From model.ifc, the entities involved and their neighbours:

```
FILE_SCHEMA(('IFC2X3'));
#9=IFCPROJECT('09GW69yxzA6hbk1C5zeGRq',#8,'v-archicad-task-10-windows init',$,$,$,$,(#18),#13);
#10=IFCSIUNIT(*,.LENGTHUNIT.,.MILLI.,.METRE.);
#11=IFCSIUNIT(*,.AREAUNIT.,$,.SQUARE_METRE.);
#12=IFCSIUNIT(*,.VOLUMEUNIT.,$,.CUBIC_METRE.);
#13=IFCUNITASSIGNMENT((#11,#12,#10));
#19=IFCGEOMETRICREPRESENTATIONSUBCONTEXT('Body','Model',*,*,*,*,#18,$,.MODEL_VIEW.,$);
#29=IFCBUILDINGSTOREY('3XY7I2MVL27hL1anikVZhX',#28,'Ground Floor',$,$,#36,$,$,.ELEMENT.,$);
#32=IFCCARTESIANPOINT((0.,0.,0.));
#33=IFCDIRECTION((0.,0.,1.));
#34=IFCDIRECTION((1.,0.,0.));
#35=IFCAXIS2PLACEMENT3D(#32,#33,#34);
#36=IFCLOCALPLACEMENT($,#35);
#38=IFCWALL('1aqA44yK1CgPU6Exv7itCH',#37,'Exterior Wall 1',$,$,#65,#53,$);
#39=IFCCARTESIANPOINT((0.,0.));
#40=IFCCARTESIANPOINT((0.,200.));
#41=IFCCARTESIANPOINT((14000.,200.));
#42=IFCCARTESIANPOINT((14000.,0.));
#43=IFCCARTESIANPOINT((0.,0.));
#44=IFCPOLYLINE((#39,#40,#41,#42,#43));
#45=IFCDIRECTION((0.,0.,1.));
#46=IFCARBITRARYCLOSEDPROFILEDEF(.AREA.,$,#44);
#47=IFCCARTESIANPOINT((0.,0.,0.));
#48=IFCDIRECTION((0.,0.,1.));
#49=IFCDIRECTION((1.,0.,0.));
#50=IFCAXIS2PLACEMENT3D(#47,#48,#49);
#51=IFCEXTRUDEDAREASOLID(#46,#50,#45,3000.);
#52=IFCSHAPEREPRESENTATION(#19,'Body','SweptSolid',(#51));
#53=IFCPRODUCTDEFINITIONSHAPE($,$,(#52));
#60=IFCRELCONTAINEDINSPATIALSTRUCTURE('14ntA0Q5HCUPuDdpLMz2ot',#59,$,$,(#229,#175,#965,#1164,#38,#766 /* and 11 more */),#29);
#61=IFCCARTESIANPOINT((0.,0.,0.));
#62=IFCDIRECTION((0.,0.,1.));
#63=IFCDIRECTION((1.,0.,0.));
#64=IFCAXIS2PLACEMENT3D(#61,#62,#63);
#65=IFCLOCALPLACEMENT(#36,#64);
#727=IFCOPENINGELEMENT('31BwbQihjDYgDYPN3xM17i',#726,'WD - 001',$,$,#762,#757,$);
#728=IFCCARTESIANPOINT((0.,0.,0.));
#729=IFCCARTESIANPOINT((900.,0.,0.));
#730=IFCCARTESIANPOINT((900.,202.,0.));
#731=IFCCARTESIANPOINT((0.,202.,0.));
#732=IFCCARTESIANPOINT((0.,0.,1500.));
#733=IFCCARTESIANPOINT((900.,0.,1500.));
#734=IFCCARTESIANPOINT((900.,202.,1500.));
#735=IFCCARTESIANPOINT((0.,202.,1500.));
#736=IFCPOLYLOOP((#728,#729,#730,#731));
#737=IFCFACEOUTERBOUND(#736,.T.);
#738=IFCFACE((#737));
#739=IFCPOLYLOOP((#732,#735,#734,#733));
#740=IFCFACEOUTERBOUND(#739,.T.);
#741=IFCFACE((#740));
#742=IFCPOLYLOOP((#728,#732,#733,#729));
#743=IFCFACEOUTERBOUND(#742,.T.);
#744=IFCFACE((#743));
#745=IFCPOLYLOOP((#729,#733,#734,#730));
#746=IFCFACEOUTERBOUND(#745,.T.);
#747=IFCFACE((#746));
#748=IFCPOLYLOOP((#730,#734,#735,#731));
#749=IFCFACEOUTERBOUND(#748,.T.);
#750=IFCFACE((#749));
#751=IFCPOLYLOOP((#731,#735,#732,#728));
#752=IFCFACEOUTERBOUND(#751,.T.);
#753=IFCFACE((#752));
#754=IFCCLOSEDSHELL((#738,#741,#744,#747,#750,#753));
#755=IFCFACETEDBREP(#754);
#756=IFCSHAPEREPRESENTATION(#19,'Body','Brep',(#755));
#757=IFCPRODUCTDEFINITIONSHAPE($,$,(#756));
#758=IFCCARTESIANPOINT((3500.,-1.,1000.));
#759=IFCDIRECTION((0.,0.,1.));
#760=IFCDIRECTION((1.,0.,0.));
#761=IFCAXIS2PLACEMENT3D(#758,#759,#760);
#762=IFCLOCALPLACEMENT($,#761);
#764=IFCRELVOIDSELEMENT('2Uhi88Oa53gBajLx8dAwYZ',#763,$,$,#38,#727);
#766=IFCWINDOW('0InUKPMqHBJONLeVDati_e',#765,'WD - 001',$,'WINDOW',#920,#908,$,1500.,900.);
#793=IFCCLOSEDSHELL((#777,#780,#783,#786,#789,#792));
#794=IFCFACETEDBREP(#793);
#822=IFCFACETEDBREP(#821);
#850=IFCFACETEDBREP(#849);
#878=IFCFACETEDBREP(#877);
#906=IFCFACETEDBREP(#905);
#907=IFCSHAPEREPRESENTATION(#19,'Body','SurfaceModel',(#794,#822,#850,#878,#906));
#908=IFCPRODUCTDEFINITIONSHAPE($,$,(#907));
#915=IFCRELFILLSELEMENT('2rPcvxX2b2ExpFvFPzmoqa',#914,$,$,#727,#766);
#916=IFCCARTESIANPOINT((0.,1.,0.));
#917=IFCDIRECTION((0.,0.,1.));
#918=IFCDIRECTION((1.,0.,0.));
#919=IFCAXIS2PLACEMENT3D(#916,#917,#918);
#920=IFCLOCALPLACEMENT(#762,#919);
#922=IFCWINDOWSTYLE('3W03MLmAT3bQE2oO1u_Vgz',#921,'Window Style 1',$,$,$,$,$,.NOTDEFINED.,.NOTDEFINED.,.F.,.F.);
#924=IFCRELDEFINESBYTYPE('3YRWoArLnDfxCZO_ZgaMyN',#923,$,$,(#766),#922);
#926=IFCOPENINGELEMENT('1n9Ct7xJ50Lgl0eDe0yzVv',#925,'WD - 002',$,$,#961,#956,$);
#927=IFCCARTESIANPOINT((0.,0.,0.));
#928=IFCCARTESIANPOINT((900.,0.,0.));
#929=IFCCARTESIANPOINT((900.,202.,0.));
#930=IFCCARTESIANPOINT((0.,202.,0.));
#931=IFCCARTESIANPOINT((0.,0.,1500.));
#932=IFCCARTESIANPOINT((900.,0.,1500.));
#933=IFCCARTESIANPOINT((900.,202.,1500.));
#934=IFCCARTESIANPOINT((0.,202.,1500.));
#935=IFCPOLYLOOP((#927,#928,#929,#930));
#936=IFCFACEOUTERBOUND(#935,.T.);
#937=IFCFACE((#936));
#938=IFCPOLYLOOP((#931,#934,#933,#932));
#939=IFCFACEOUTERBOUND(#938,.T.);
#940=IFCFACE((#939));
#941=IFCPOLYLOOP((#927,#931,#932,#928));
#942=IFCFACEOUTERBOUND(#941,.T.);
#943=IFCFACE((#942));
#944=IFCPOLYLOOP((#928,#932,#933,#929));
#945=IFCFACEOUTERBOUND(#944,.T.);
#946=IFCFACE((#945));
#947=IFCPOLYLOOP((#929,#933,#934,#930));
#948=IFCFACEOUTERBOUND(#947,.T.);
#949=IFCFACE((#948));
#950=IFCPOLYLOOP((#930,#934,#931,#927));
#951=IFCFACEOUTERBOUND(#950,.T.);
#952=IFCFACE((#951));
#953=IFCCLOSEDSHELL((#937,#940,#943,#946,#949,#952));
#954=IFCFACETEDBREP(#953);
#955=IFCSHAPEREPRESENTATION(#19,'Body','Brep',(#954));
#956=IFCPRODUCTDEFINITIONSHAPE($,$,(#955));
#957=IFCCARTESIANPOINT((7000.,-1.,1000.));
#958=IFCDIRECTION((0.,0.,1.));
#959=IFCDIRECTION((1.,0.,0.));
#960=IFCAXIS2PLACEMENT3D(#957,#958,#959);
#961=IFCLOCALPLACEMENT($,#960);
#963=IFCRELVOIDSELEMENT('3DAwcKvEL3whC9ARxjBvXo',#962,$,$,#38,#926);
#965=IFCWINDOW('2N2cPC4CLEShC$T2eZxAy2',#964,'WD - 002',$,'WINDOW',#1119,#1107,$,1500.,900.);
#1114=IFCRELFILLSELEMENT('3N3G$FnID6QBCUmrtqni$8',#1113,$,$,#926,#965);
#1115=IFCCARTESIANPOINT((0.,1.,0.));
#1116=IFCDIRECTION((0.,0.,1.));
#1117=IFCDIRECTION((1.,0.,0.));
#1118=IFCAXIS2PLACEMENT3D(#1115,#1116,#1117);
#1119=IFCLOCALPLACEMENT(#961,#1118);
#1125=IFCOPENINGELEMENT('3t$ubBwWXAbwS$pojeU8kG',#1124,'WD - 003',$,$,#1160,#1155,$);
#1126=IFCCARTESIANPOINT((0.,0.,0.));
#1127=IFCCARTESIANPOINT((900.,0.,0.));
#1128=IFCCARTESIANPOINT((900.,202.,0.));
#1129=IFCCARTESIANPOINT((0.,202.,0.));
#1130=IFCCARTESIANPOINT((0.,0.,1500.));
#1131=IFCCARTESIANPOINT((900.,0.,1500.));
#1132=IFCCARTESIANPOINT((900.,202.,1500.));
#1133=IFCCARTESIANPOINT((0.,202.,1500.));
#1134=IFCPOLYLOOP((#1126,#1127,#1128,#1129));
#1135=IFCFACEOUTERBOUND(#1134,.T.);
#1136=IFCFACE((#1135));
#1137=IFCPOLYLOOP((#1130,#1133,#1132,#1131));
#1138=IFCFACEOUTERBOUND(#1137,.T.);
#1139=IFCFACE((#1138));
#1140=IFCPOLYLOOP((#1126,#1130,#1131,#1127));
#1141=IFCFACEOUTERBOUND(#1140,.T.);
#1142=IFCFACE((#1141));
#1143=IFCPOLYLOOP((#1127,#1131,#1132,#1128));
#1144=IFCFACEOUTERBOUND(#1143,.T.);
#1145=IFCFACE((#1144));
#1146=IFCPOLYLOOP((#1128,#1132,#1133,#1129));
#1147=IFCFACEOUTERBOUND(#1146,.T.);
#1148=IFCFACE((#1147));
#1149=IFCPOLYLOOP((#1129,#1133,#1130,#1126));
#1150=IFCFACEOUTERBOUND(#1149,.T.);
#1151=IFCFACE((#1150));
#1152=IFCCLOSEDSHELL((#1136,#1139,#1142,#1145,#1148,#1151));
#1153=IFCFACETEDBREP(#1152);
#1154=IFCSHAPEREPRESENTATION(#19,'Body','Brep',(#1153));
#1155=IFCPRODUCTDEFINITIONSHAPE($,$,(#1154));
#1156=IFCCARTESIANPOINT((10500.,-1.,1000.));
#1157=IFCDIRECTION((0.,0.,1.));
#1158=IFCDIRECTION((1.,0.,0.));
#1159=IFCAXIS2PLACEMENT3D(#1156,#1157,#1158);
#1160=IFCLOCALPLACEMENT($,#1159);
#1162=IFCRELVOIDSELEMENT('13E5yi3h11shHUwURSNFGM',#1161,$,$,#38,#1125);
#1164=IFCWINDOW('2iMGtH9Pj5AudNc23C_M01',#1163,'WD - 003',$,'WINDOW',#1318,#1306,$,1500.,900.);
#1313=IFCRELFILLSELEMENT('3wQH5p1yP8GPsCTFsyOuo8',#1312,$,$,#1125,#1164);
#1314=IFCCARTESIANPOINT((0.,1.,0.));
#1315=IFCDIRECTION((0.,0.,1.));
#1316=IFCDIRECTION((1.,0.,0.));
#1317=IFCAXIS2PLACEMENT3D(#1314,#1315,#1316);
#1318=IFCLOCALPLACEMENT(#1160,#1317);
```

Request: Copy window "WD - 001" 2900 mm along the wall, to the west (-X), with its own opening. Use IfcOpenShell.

```python
import ifcopenshell
import ifcopenshell.api.feature
import ifcopenshell.api.geometry
import ifcopenshell.api.root
import ifcopenshell.geom
import ifcopenshell.util.element
import ifcopenshell.util.placement
import ifcopenshell.util.shape
import ifcopenshell.util.unit

model = ifcopenshell.open("model.ifc")
unit_scale = ifcopenshell.util.unit.calculate_unit_scale(model)
settings = ifcopenshell.geom.settings()


def volume(element):
    """Net volume in cubic metres, openings subtracted."""
    shape = ifcopenshell.geom.create_shape(settings, element)
    return ifcopenshell.util.shape.get_volume(shape.geometry)


window = model.by_guid("0InUKPMqHBJONLeVDati_e")
opening = window.FillsVoids[0].RelatingOpeningElement
wall = opening.VoidsElements[0].RelatingBuildingElement
before = volume(wall)
shift = ifcopenshell.util.placement.get_local_placement(wall.ObjectPlacement)[:3, 0] * -2.9 / unit_scale

# copy_class copies the void relationship, type, container and properties, but no geometry.
new_opening = ifcopenshell.api.root.copy_class(model, product=opening)
new_opening.Representation = ifcopenshell.util.element.copy_deep(
    model, opening.Representation, exclude=["IfcGeometricRepresentationContext", "IfcRepresentationMap"]
)
new_window = ifcopenshell.api.root.copy_class(model, product=window)
new_window.Representation = ifcopenshell.util.element.copy_deep(
    model, window.Representation, exclude=["IfcGeometricRepresentationContext", "IfcRepresentationMap"]
)
fills = ifcopenshell.api.feature.add_filling(model, opening=new_opening, element=new_window)
fills.OwnerHistory = new_window.OwnerHistory  # required in IFC2X3

for old, new in ((opening, new_opening), (window, new_window)):
    matrix = ifcopenshell.util.placement.get_local_placement(old.ObjectPlacement)
    matrix[:3, 3] += shift
    ifcopenshell.api.geometry.edit_object_placement(model, product=new, matrix=matrix, is_si=False)

after = volume(wall)

print(f"wall volume {before:.3f} -> {after:.3f} m3")

model.write("model_updated.ifc")
```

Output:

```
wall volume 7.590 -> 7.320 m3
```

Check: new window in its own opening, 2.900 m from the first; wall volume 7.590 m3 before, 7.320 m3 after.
